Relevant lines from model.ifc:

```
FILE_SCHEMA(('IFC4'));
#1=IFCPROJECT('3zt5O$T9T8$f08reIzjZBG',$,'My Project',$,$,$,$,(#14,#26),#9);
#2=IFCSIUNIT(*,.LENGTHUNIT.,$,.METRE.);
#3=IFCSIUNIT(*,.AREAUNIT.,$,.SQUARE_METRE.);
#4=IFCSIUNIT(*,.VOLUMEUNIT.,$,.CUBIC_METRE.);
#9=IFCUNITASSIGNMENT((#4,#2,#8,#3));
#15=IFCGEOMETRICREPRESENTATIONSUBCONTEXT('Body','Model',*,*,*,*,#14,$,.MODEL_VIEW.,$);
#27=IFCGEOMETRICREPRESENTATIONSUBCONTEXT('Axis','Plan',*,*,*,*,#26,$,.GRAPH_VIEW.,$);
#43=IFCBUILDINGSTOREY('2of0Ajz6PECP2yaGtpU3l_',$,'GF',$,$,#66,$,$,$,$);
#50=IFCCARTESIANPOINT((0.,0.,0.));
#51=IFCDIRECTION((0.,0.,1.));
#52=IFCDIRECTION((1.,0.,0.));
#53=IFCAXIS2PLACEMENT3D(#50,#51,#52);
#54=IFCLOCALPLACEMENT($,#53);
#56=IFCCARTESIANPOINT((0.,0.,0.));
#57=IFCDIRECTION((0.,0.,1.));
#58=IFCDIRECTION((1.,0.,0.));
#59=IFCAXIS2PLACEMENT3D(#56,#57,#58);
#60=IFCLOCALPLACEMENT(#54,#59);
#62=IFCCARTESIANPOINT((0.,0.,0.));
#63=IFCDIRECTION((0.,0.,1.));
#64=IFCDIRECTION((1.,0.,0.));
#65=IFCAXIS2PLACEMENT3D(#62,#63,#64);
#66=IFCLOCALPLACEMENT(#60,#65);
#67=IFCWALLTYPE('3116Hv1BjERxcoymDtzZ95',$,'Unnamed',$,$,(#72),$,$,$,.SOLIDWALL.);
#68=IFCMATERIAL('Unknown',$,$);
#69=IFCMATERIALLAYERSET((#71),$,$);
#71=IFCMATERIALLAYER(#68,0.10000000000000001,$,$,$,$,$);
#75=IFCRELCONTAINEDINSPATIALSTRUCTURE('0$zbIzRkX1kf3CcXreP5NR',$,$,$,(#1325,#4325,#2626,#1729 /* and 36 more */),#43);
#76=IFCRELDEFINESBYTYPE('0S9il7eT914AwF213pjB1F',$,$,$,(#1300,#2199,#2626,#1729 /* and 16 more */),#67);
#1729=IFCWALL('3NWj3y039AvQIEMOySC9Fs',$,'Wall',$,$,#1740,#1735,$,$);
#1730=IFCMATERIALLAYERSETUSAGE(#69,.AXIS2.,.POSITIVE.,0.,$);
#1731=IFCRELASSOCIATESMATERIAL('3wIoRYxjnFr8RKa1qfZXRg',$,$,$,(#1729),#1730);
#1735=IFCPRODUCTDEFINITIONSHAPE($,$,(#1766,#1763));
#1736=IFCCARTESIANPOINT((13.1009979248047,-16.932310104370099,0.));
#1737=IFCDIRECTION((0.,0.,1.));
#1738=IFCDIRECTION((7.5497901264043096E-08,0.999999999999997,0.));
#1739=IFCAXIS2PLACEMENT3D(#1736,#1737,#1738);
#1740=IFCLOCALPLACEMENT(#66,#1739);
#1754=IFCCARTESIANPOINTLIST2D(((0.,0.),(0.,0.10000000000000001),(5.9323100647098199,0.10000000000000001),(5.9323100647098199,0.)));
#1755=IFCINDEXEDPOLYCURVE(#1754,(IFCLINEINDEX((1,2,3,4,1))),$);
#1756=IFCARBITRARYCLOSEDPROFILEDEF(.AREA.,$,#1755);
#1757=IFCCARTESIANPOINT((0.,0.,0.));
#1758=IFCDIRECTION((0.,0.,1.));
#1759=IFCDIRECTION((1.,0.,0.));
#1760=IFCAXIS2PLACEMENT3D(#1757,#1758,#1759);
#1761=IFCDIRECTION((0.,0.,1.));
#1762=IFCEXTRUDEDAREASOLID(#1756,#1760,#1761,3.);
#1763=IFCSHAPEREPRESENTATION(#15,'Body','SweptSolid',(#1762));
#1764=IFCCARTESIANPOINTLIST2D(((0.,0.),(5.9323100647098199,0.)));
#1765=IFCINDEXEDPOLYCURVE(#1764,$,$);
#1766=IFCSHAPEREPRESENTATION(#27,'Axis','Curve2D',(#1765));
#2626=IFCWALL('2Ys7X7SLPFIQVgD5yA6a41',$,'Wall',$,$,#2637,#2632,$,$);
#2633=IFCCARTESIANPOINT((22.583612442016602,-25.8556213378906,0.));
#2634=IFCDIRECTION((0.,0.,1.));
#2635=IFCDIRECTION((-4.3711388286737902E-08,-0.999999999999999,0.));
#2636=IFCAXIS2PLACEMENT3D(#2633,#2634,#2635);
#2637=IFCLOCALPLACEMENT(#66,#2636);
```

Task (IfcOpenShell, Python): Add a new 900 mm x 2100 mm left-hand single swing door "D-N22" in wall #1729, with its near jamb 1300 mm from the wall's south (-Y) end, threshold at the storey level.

```python
import numpy as np
import ifcopenshell
import ifcopenshell.api.feature
import ifcopenshell.api.geometry
import ifcopenshell.api.root
import ifcopenshell.api.spatial
import ifcopenshell.geom
import ifcopenshell.util.element
import ifcopenshell.util.placement
import ifcopenshell.util.representation
import ifcopenshell.util.shape
import ifcopenshell.util.unit

model = ifcopenshell.open("model.ifc")
unit_scale = ifcopenshell.util.unit.calculate_unit_scale(model)
settings = ifcopenshell.geom.settings()


def volume(element):
    """Net volume in cubic metres, openings subtracted."""
    shape = ifcopenshell.geom.create_shape(settings, element)
    return ifcopenshell.util.shape.get_volume(shape.geometry)


wall = model.by_guid("3NWj3y039AvQIEMOySC9Fs")
storey = ifcopenshell.util.element.get_container(wall, ifc_class="IfcBuildingStorey")
context = ifcopenshell.util.representation.get_context(model, "Model", "Body", "MODEL_VIEW")
before = volume(wall)

width, height, from_end, sill = 0.9, 2.1, 1.3, 0.0  # metres

# The wall runs along its own X axis, and the end named is its -X end.
wall_shape = ifcopenshell.geom.create_shape(settings, wall)
x, y, z = ifcopenshell.util.shape.get_vertices(wall_shape.geometry).T
start = x.min() + from_end
face, thickness = float(y.min()), float(y.max() - y.min())
wall_matrix = ifcopenshell.util.placement.get_local_placement(wall.ObjectPlacement)
level = ifcopenshell.util.placement.get_local_placement(storey.ObjectPlacement)[2, 3]


def in_wall(x, y):
    """Placement at x, y metres in the wall's axes, at sill height."""
    matrix = wall_matrix.copy()
    matrix[:, 3] = wall_matrix @ np.array([x / unit_scale, y / unit_scale, 0.0, 1.0])
    matrix[2, 3] = level + sill / unit_scale
    return matrix


# Opening: a box that overshoots both wall faces by 50 mm.
opening = ifcopenshell.api.root.create_entity(model, ifc_class="IfcOpeningElement", predefined_type="OPENING")
box = ifcopenshell.api.geometry.add_wall_representation(
    model, context=context, length=width, height=height, thickness=thickness + 0.1
)
ifcopenshell.api.geometry.assign_representation(model, product=opening, representation=box)
ifcopenshell.api.geometry.edit_object_placement(model, product=opening, matrix=in_wall(start, face - 0.05), is_si=False)
ifcopenshell.api.feature.add_feature(model, feature=opening, element=wall)

door = ifcopenshell.api.root.create_entity(model, ifc_class="IfcDoor", name="D-N22", predefined_type="DOOR")
door.OverallWidth, door.OverallHeight = width / unit_scale, height / unit_scale
door.OperationType = "SINGLE_SWING_LEFT"
body = ifcopenshell.api.geometry.add_door_representation(
    model,
    context=context,
    overall_width=door.OverallWidth,
    overall_height=door.OverallHeight,
    operation_type="SINGLE_SWING_LEFT",
    lining_properties={"LiningDepth": thickness / unit_scale, "ThresholdDepth": thickness / unit_scale},
)
ifcopenshell.api.geometry.assign_representation(model, product=door, representation=body)
ifcopenshell.api.spatial.assign_container(model, products=[door], relating_structure=storey)
ifcopenshell.api.feature.add_filling(model, opening=opening, element=door)

# The lining spans the wall, so the door starts at the wall face.
ifcopenshell.api.geometry.edit_object_placement(model, product=door, matrix=in_wall(start, face), is_si=False)

after = volume(wall)

print(f"wall volume {before:.3f} -> {after:.3f} m3")

model.write("model_rev.ifc")
```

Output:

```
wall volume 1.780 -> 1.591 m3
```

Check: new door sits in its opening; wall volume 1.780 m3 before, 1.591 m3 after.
